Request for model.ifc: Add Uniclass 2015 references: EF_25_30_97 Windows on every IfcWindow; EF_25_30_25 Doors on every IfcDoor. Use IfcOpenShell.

First a look at what the model holds.

```python
import ifcopenshell

model = ifcopenshell.open("model.ifc")
print(model.schema)
print("classifications:", [c.Name for c in model.by_type("IfcClassification")])
for ifc_class in ("IfcDoor", "IfcRoof", "IfcStair", "IfcWall", "IfcWindow"):
    print(ifc_class, len(model.by_type(ifc_class)))
```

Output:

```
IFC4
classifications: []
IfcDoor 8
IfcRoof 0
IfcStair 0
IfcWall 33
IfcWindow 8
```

```python
import ifcopenshell
import ifcopenshell.api.classification

model = ifcopenshell.open("model.ifc")

system = ifcopenshell.api.classification.add_classification(model, classification="Uniclass 2015")

codes = {
    "IfcWindow": ("EF_25_30_97", "Windows"),
    "IfcDoor": ("EF_25_30_25", "Doors"),
}
for ifc_class, (code, name) in codes.items():
    products = model.by_type(ifc_class)
    ifcopenshell.api.classification.add_reference(
        model, products=products, classification=system, identification=code, name=name
    )
    print(code, len(products))

model.write("model-out.ifc")
```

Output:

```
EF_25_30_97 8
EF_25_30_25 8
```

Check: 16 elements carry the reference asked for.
